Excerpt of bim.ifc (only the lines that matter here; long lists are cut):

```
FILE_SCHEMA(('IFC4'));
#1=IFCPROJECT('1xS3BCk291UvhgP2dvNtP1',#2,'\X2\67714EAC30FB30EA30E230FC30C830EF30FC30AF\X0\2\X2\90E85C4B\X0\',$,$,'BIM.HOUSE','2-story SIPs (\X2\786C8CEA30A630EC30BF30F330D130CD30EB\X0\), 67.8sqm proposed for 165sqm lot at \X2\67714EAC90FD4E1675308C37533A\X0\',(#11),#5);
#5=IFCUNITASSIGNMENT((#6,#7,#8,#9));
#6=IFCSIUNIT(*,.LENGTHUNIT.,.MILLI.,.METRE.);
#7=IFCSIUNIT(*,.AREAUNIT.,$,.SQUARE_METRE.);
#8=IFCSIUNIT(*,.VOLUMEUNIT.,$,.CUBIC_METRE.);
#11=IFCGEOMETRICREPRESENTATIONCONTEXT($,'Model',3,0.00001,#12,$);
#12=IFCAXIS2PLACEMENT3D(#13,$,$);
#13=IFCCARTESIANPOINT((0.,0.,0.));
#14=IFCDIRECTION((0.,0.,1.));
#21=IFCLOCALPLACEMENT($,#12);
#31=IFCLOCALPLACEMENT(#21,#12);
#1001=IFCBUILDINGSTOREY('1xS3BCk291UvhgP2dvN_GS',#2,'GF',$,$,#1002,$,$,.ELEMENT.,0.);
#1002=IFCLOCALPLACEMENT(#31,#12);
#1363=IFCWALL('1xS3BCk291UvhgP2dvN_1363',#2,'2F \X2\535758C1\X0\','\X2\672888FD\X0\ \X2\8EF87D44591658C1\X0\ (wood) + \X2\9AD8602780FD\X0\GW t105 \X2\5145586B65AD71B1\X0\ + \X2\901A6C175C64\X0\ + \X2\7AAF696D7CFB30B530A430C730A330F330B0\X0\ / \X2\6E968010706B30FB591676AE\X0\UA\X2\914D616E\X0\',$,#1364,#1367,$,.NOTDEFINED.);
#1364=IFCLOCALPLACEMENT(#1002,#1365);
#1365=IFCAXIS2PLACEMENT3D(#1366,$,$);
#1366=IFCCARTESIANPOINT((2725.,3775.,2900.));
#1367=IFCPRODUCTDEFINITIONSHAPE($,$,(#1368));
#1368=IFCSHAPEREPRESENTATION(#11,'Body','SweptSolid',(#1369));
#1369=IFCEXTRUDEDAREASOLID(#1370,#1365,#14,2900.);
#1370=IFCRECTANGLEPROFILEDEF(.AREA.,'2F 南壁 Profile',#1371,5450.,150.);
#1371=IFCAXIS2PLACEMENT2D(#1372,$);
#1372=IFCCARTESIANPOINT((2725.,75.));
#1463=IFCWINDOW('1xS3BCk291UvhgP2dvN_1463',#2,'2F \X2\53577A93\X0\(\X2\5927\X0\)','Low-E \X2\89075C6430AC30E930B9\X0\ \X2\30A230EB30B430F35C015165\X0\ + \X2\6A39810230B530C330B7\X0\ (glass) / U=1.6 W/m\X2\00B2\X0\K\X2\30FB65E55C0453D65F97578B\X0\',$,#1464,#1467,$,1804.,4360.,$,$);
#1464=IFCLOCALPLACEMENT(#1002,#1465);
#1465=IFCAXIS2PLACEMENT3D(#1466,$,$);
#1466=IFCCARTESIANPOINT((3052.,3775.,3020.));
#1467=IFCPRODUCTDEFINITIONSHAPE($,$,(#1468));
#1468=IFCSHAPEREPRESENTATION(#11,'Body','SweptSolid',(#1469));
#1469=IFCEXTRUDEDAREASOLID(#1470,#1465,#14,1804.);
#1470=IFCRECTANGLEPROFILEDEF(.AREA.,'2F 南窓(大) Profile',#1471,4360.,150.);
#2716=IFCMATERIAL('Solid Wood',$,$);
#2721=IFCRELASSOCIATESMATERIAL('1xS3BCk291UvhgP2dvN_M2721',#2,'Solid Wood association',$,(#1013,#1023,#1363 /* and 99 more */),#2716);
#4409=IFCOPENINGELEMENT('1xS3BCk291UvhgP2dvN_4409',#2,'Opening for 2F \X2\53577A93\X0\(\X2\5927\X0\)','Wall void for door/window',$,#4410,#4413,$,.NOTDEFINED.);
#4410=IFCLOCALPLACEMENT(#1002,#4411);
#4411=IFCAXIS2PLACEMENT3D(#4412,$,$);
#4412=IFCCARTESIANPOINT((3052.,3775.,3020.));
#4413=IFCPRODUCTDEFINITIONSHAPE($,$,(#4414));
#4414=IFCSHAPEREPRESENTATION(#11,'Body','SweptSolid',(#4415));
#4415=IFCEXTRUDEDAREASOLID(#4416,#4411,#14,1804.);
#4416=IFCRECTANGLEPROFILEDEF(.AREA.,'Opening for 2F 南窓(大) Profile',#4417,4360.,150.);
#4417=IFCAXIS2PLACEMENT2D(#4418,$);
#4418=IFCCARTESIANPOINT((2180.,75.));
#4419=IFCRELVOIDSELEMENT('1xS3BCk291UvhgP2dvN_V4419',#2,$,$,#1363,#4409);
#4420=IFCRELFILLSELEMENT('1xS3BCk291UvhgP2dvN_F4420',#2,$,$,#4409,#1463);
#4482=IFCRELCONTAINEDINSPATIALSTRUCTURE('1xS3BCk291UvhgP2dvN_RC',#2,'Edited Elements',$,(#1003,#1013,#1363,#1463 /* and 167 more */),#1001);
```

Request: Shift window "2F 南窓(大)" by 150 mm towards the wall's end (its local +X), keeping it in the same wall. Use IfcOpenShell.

```python
import ifcopenshell
import ifcopenshell.api.geometry
import ifcopenshell.util.placement
import ifcopenshell.util.unit

model = ifcopenshell.open("bim.ifc")
unit_scale = ifcopenshell.util.unit.calculate_unit_scale(model)

window = model.by_guid("1xS3BCk291UvhgP2dvN_1463")
opening = window.FillsVoids[0].RelatingOpeningElement
wall = opening.VoidsElements[0].RelatingBuildingElement

wall_matrix = ifcopenshell.util.placement.get_local_placement(wall.ObjectPlacement)
shift = wall_matrix[:3, 0] * 0.15 / unit_scale
before = ifcopenshell.util.placement.get_local_placement(window.ObjectPlacement)[:3, 3].copy()

# The window is not placed relative to its opening, so move both.
for product in (opening, window):
    matrix = ifcopenshell.util.placement.get_local_placement(product.ObjectPlacement)
    matrix[:3, 3] += shift
    ifcopenshell.api.geometry.edit_object_placement(model, product=product, matrix=matrix, is_si=False)

after = ifcopenshell.util.placement.get_local_placement(window.ObjectPlacement)[:3, 3]
print("window moved by", (after - before).round(3) + 0.0)

model.write("bim_rev.ifc")
```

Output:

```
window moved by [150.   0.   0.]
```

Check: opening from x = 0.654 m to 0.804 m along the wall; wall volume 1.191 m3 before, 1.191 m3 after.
